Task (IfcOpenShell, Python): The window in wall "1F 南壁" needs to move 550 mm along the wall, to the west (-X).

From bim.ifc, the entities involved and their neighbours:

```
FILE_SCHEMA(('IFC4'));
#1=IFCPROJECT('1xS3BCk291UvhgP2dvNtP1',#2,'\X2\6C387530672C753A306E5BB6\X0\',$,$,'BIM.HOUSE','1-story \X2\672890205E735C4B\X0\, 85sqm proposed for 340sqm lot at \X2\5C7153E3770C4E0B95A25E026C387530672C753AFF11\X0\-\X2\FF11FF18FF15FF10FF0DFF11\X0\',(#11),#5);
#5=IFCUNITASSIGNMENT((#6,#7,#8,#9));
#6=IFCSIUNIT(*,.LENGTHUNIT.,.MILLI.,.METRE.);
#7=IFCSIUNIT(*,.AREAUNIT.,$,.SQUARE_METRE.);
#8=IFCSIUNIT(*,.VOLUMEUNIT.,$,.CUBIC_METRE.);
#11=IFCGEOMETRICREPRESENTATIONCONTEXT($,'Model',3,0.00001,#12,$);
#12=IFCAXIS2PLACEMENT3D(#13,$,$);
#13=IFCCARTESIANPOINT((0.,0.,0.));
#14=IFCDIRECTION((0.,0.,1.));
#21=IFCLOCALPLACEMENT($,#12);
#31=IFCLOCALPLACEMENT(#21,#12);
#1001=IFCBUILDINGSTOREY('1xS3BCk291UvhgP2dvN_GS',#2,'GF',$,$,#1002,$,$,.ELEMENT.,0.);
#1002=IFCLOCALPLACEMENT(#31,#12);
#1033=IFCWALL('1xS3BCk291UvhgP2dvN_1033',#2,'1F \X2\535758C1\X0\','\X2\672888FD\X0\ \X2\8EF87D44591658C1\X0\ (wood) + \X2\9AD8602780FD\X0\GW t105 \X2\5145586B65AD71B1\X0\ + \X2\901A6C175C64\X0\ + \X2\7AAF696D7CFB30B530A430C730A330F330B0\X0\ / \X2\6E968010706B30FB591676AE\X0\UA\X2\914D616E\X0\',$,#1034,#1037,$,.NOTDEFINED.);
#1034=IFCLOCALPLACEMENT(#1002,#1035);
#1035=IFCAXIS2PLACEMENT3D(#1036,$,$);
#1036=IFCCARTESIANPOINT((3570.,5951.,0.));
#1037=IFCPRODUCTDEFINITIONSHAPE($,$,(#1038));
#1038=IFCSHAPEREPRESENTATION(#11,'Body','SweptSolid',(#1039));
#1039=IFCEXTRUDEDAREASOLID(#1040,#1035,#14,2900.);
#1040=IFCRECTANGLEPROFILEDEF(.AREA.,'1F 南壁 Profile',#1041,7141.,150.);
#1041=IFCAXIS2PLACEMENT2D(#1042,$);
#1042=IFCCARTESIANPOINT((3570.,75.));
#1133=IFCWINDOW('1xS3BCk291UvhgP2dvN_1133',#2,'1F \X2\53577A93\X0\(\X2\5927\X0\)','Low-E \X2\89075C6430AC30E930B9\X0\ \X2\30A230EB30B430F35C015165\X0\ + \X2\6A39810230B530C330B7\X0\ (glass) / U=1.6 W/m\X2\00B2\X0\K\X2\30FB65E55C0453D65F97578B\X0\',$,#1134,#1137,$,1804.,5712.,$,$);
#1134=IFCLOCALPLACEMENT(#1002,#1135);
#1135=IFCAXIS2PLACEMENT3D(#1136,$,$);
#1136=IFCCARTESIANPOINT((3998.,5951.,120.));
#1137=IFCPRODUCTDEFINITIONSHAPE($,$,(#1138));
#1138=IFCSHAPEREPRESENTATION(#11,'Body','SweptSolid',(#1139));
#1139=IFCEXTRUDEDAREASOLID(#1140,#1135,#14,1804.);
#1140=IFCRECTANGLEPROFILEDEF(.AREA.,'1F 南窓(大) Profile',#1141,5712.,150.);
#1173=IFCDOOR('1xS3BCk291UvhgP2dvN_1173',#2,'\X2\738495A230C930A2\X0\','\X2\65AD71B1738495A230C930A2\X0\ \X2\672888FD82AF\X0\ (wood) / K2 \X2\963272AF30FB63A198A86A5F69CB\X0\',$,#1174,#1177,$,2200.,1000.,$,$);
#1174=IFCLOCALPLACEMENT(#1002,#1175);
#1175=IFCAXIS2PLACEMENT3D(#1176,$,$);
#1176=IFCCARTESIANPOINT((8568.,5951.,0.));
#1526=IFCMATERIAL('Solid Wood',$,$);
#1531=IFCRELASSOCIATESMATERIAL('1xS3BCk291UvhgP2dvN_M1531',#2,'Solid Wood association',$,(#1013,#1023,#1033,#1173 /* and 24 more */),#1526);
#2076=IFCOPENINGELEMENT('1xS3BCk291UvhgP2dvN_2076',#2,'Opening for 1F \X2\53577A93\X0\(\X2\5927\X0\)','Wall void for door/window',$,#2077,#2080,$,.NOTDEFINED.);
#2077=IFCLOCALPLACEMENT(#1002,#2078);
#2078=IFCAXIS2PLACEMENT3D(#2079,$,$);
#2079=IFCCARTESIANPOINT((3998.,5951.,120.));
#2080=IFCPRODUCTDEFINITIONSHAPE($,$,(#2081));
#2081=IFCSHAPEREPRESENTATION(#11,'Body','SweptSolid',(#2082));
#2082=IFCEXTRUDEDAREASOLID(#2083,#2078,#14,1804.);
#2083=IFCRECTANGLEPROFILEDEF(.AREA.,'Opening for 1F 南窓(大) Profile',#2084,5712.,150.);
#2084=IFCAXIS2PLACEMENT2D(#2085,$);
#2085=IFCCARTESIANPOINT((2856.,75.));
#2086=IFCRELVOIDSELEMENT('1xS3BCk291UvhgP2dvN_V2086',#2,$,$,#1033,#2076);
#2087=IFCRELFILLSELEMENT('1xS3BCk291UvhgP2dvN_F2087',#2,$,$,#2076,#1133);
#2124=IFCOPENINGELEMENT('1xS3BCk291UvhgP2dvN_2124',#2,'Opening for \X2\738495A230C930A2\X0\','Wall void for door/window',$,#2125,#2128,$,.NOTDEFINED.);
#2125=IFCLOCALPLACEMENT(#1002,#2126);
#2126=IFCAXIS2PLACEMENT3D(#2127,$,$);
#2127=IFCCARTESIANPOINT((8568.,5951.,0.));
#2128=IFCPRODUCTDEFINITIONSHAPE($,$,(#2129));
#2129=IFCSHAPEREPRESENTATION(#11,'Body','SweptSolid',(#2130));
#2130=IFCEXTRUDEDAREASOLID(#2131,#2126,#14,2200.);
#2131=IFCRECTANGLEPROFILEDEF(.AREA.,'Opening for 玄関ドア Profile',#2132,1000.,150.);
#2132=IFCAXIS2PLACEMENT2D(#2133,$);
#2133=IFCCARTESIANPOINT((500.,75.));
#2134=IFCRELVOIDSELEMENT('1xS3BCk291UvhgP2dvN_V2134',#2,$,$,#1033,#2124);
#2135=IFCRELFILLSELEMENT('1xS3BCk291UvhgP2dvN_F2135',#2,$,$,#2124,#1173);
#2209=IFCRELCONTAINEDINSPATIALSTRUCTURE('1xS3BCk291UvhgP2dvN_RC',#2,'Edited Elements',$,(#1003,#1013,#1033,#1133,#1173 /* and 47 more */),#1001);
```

```python
import ifcopenshell
import ifcopenshell.api.geometry
import ifcopenshell.util.placement

model = ifcopenshell.open("bim.ifc")

window = model.by_guid("1xS3BCk291UvhgP2dvN_1133")
opening = window.FillsVoids[0].RelatingOpeningElement
wall = opening.VoidsElements[0].RelatingBuildingElement

wall_matrix = ifcopenshell.util.placement.get_local_placement(wall.ObjectPlacement)
shift = wall_matrix[:3, 0] * -550.0
before = ifcopenshell.util.placement.get_local_placement(window.ObjectPlacement)[:3, 3].copy()

# The window is not placed relative to its opening, so move both.
for product in (opening, window):
    matrix = ifcopenshell.util.placement.get_local_placement(product.ObjectPlacement)
    matrix[:3, 3] += shift
    ifcopenshell.api.geometry.edit_object_placement(model, product=product, matrix=matrix, is_si=False)

after = ifcopenshell.util.placement.get_local_placement(window.ObjectPlacement)[:3, 3]
print("window moved by", (after - before).round(3) + 0.0)

model.write("bim_updated.ifc")
```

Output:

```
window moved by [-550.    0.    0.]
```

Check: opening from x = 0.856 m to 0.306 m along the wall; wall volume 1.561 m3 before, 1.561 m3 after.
